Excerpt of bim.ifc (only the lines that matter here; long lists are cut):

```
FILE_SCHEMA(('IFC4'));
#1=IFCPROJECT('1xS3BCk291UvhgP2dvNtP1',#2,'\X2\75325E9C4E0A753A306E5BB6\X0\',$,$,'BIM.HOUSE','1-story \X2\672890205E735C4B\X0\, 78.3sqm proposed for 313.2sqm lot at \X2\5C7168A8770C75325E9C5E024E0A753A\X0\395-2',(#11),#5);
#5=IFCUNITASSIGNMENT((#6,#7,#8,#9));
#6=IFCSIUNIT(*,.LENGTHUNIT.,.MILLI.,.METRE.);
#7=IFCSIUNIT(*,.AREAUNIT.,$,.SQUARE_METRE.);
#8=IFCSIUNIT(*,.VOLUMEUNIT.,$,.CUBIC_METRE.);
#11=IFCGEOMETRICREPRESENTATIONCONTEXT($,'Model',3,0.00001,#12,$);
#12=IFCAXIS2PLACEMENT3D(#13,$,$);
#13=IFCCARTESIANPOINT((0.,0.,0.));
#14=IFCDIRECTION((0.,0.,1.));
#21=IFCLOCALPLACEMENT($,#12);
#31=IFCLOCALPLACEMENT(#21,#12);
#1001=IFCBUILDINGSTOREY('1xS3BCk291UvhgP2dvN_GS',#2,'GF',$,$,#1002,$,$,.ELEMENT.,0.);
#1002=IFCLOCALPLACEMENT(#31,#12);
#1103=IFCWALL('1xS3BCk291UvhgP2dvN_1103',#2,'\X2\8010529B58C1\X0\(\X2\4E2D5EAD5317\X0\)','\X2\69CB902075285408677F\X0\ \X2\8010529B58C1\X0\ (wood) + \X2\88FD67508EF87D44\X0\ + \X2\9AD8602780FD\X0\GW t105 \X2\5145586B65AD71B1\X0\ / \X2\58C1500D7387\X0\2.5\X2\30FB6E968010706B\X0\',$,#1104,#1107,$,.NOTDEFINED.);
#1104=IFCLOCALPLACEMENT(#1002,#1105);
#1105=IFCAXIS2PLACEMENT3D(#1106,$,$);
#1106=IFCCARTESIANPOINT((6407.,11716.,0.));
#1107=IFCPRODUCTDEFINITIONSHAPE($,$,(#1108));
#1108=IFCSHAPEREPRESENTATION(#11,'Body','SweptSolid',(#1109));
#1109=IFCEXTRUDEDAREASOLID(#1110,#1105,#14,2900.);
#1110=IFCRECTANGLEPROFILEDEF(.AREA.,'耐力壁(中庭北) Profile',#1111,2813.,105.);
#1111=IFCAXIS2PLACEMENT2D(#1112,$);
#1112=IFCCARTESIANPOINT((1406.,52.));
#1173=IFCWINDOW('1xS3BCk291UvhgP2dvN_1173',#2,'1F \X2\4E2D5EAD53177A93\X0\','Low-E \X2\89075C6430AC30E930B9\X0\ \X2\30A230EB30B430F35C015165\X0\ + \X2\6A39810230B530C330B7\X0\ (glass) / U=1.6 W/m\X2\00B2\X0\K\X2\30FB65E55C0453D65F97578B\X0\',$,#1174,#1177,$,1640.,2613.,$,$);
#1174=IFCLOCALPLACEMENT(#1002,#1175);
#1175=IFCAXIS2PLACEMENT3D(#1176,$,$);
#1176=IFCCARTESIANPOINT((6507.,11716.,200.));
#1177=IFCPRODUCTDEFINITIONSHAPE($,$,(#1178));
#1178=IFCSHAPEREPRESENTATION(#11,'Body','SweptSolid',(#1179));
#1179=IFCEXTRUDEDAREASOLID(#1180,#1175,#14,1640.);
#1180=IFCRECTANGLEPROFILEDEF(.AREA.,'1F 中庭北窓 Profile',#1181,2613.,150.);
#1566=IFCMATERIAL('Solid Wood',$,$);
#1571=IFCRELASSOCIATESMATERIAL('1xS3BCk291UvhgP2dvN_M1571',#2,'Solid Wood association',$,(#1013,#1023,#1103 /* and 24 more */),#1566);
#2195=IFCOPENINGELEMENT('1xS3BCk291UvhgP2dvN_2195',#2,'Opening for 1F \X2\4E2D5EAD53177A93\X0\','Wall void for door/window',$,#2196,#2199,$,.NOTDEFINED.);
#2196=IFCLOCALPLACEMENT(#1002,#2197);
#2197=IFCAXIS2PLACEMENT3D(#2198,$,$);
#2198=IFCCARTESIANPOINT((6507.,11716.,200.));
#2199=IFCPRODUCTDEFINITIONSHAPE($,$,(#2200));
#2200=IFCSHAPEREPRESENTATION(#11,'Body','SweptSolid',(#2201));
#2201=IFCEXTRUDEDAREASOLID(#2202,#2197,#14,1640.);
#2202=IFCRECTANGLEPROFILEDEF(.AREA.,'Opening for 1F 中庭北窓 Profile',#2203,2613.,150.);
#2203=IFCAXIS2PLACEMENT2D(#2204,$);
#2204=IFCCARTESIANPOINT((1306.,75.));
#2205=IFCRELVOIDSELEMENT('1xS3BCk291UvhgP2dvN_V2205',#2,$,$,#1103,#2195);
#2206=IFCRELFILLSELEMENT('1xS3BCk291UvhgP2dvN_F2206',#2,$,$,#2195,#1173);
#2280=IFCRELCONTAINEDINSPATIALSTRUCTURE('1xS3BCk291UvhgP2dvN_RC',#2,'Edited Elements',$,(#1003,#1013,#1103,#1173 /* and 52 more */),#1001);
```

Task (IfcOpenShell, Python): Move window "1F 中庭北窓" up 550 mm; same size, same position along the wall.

```python
import numpy as np
import ifcopenshell
import ifcopenshell.api.geometry
import ifcopenshell.util.placement
import ifcopenshell.util.unit

model = ifcopenshell.open("bim.ifc")
unit_scale = ifcopenshell.util.unit.calculate_unit_scale(model)

window = model.by_guid("1xS3BCk291UvhgP2dvN_1173")
opening = window.FillsVoids[0].RelatingOpeningElement
dz = 550.0

shift = np.array([0.0, 0.0, dz])
# The window is not placed relative to its opening, so move both.
for product in (opening, window):
    matrix = ifcopenshell.util.placement.get_local_placement(product.ObjectPlacement)
    matrix[:3, 3] += shift
    ifcopenshell.api.geometry.edit_object_placement(model, product=product, matrix=matrix, is_si=False)

print(f"moved by {dz * unit_scale:+.3f} m")

model.write("bim_edited.ifc")
```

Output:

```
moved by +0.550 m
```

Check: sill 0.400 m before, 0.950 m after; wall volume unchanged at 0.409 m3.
